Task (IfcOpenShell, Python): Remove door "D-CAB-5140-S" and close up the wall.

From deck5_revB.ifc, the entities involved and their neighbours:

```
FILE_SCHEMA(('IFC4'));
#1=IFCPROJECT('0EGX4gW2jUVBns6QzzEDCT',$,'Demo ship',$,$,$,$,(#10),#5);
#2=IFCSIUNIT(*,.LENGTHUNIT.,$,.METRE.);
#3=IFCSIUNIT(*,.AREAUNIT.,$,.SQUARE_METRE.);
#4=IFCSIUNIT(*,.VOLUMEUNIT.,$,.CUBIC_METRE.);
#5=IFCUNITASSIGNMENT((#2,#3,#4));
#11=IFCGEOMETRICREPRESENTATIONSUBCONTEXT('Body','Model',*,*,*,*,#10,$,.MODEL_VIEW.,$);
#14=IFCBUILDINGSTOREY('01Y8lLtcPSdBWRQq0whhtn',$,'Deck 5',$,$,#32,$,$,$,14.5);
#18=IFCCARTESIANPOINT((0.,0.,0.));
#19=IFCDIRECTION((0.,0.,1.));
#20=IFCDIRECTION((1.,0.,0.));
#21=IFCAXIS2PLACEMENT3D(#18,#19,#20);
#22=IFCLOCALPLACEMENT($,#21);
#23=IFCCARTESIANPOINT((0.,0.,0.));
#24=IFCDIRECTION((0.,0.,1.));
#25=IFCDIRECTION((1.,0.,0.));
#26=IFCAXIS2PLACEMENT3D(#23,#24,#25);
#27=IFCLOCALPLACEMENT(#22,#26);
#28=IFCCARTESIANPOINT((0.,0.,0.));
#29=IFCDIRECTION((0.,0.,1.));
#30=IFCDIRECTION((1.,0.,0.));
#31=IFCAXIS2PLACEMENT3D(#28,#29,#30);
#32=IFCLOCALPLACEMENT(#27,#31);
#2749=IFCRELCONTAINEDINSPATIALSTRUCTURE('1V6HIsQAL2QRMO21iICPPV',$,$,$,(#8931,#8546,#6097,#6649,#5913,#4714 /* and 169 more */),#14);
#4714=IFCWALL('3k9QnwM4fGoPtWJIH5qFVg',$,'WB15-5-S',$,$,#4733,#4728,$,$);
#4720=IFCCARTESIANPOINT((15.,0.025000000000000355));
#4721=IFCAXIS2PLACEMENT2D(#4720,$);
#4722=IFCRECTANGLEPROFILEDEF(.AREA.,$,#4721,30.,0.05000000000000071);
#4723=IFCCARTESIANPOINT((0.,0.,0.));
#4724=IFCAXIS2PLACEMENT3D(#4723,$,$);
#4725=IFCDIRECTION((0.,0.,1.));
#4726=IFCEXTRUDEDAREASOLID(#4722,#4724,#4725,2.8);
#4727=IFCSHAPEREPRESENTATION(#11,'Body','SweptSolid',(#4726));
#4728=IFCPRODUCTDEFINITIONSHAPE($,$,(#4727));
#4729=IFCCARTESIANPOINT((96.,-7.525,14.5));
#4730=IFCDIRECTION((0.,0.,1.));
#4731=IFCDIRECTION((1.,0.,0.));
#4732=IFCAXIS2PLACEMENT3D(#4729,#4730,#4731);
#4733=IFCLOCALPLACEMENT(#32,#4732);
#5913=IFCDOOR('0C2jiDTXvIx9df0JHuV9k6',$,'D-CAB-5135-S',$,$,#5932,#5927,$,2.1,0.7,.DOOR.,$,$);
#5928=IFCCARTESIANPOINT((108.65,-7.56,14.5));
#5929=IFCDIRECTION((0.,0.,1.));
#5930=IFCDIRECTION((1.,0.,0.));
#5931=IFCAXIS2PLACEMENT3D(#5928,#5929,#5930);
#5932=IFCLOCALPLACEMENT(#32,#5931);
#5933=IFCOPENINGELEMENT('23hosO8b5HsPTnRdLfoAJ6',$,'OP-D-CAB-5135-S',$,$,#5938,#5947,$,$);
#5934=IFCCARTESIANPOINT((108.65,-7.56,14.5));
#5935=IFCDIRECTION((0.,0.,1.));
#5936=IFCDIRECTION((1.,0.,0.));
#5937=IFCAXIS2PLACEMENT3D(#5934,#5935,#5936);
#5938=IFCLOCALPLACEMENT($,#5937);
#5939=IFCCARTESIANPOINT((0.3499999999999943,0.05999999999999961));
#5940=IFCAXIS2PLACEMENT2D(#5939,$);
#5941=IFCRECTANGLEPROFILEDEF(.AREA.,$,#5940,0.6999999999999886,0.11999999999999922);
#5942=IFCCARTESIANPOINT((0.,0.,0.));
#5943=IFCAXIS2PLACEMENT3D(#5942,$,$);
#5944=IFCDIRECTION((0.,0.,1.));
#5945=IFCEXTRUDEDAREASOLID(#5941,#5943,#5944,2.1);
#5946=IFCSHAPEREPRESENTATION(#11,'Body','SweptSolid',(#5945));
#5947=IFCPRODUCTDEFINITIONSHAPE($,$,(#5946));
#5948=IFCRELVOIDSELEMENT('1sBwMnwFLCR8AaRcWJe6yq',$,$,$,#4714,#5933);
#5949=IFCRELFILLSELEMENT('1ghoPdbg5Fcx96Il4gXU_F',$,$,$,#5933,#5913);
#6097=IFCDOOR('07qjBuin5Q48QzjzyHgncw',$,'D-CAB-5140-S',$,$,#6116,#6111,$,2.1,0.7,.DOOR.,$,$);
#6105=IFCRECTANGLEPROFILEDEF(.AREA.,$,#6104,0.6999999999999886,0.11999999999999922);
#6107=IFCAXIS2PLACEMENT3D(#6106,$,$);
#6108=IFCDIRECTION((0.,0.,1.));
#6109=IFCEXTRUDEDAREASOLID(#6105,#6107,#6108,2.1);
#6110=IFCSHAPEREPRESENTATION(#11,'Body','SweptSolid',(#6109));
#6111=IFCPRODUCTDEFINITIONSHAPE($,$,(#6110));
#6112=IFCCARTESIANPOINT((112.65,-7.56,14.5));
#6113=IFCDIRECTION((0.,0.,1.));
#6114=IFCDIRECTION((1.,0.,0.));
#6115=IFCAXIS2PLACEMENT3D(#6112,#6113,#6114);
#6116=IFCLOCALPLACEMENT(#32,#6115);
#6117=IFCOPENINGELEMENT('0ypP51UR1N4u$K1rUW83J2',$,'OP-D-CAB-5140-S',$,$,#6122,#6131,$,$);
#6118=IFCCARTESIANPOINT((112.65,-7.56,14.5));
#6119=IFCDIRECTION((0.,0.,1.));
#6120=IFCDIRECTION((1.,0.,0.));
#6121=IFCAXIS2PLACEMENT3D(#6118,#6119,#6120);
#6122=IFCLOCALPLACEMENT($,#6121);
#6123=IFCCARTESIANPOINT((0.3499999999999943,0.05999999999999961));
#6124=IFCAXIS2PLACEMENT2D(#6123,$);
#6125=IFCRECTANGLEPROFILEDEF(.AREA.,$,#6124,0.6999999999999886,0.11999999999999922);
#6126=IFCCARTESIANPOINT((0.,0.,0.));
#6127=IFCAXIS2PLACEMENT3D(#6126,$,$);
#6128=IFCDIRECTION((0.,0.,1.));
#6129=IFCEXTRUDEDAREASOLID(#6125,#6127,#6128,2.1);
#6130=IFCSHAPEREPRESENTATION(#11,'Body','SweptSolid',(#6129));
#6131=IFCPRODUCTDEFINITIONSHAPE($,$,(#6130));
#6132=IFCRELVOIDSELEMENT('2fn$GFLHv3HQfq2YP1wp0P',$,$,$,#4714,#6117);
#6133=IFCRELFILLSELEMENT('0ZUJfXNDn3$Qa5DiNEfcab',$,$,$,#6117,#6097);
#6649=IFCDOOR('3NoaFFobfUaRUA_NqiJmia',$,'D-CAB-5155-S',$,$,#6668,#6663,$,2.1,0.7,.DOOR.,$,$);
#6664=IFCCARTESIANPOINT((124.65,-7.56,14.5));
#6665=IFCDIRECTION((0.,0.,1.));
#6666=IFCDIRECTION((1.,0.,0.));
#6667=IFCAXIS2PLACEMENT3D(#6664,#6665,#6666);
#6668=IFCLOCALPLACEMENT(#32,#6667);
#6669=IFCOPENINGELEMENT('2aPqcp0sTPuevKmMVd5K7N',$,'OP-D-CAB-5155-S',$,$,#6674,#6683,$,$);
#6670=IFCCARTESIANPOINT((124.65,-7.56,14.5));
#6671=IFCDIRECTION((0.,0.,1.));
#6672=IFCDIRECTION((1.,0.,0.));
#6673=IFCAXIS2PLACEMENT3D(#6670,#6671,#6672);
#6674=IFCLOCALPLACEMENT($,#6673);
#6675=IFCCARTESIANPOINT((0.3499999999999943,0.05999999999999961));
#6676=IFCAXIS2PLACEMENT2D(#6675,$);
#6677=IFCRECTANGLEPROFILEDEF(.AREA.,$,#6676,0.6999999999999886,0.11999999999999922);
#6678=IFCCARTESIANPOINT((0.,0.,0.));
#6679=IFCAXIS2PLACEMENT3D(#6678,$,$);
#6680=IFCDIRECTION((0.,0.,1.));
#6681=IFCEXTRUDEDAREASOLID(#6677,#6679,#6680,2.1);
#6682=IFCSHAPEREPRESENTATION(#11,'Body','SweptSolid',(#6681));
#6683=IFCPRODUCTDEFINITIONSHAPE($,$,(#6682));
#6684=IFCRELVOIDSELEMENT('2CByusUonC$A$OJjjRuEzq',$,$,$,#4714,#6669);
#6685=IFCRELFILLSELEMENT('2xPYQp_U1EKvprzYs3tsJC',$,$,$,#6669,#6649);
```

```python
import ifcopenshell
import ifcopenshell.api.feature
import ifcopenshell.api.root
import ifcopenshell.geom
import ifcopenshell.util.shape

model = ifcopenshell.open("deck5_revB.ifc")
settings = ifcopenshell.geom.settings()


def volume(element):
    """Net volume in cubic metres, openings subtracted."""
    shape = ifcopenshell.geom.create_shape(settings, element)
    return ifcopenshell.util.shape.get_volume(shape.geometry)


door = model.by_guid("07qjBuin5Q48QzjzyHgncw")
opening = door.FillsVoids[0].RelatingOpeningElement
wall = opening.VoidsElements[0].RelatingBuildingElement
before = volume(wall)

ifcopenshell.api.root.remove_product(model, product=door)
ifcopenshell.api.feature.remove_feature(model, feature=opening)

after = volume(wall)

print(f"wall volume {before:.3f} -> {after:.3f} m3")

model.write("deck5_revB_updated.ifc")
```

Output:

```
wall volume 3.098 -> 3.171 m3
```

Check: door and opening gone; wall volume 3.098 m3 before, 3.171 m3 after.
